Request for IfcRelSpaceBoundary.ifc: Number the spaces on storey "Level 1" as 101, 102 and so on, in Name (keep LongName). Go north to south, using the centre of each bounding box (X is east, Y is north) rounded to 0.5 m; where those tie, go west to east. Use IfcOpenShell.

First a look at what the model holds.

```python
import ifcopenshell
import ifcopenshell.util.element
import ifcopenshell.util.placement

model = ifcopenshell.open("IfcRelSpaceBoundary.ifc")
print(model.schema)
storey = next(s for s in model.by_type("IfcBuildingStorey") if s.Name == "Level 1")
spaces = [e for e in ifcopenshell.util.element.get_decomposition(storey) if e.is_a("IfcSpace")]
for e in sorted(spaces, key=lambda e: e.id()):
    origin = ifcopenshell.util.placement.get_local_placement(e.ObjectPlacement)[:3, 3]
    print(e.id(), e.Name, e.LongName, origin.round(2) + 0.0, sep=" | ")
```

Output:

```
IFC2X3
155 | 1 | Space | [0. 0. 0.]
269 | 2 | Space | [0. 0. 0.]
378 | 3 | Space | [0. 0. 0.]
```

```python
import ifcopenshell
import ifcopenshell.geom
import ifcopenshell.util.element
import ifcopenshell.util.shape

model = ifcopenshell.open("IfcRelSpaceBoundary.ifc")
settings = ifcopenshell.geom.settings()
settings.set("use-world-coords", True)


def centre(element):
    shape = ifcopenshell.geom.create_shape(settings, element)
    return ifcopenshell.util.shape.get_bbox_centroid(shape.geometry)


storey = next(s for s in model.by_type("IfcBuildingStorey") if s.Name == "Level 1")
spaces = [e for e in ifcopenshell.util.element.get_decomposition(storey) if e.is_a("IfcSpace")]

# Insertion points can sit at a corner or the storey origin, so sort by the geometry (in metres).
centres = {e: centre(e) for e in spaces}
spaces.sort(key=lambda e: (-round(centres[e][1] / 0.5), centres[e][0]))

for i, e in enumerate(spaces, start=1):
    number = f"1{i:02d}"
    e.Name = number
    print(e.id(), number)

model.write("IfcRelSpaceBoundary_v2.ifc")
```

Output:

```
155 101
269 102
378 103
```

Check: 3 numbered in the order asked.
